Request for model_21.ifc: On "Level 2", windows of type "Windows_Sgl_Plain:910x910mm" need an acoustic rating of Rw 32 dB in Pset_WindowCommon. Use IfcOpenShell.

First a look at what the model holds.

```python
import ifcopenshell
import ifcopenshell.util.element

model = ifcopenshell.open("model_21.ifc")
print(model.schema)
storey = next(s for s in model.by_type("IfcBuildingStorey") if s.Name == "Level 2")
windows = [e for e in ifcopenshell.util.element.get_decomposition(storey) if e.is_a("IfcWindow")]
seen = {}
for e in windows:
    element_type = ifcopenshell.util.element.get_type(e)
    key = (element_type.Name if element_type != e and element_type else None, ifcopenshell.util.element.get_pset(e, "Pset_WindowCommon", "AcousticRating"))
    seen[key] = seen.get(key, 0) + 1
for (name, value), count in sorted(seen.items(), key=str):
    print(count, "x", name, "|", value)
```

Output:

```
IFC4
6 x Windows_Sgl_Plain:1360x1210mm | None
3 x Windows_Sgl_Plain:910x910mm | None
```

```python
import ifcopenshell
import ifcopenshell.api.pset
import ifcopenshell.util.element

model = ifcopenshell.open("model_21.ifc")

storey = next(s for s in model.by_type("IfcBuildingStorey") if s.Name == "Level 2")
windows = [e for e in ifcopenshell.util.element.get_decomposition(storey) if e.is_a("IfcWindow")]

count = 0
for e in windows:
    element_type = ifcopenshell.util.element.get_type(e)
    if element_type in (None, e) or element_type.Name != "Windows_Sgl_Plain:910x910mm":
        continue
    # add_pset returns the element's existing set when there is one.
    pset = ifcopenshell.api.pset.add_pset(model, product=e, name="Pset_WindowCommon")
    ifcopenshell.api.pset.edit_pset(model, pset=pset, properties={"AcousticRating": "Rw 32 dB"})
    count += 1

print(count, "windows updated")

model.write("model_21_v2.ifc")
```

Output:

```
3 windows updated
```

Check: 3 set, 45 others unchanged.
